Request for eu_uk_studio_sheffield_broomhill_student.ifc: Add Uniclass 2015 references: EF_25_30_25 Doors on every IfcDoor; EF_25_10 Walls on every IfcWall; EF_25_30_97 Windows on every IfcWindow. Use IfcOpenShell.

First a look at what the model holds.

```python
import ifcopenshell

model = ifcopenshell.open("eu_uk_studio_sheffield_broomhill_student.ifc")
print(model.schema)
print("classifications:", [c.Name for c in model.by_type("IfcClassification")])
for ifc_class in ("IfcDoor", "IfcRoof", "IfcStair", "IfcWall", "IfcWindow"):
    print(ifc_class, len(model.by_type(ifc_class)))
```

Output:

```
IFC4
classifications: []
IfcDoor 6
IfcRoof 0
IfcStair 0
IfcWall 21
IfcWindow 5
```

```python
import ifcopenshell
import ifcopenshell.api.classification

model = ifcopenshell.open("eu_uk_studio_sheffield_broomhill_student.ifc")

system = ifcopenshell.api.classification.add_classification(model, classification="Uniclass 2015")

codes = {
    "IfcDoor": ("EF_25_30_25", "Doors"),
    "IfcWall": ("EF_25_10", "Walls"),
    "IfcWindow": ("EF_25_30_97", "Windows"),
}
for ifc_class, (code, name) in codes.items():
    products = model.by_type(ifc_class)
    ifcopenshell.api.classification.add_reference(
        model, products=products, classification=system, identification=code, name=name
    )
    print(code, len(products))

model.write("eu_uk_studio_sheffield_broomhill_student-out.ifc")
```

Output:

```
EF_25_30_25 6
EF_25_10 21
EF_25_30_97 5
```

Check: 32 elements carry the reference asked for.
